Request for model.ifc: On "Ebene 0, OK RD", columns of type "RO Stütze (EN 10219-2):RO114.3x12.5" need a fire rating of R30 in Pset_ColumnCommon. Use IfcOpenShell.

First a look at what the model holds.

```python
import ifcopenshell
import ifcopenshell.util.element

model = ifcopenshell.open("model.ifc")
print(model.schema)
storey = next(s for s in model.by_type("IfcBuildingStorey") if s.Name == "Ebene 0, OK RD")
columns = [e for e in ifcopenshell.util.element.get_decomposition(storey) if e.is_a("IfcColumn")]
seen = {}
for e in columns:
    element_type = ifcopenshell.util.element.get_type(e)
    key = (element_type.Name if element_type != e and element_type else None, ifcopenshell.util.element.get_pset(e, "Pset_ColumnCommon", "FireRating"))
    seen[key] = seen.get(key, 0) + 1
for (name, value), count in sorted(seen.items(), key=str):
    print(count, "x", name, "|", value)
```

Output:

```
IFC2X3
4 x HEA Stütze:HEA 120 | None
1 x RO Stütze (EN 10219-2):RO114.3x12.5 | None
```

```python
import ifcopenshell
import ifcopenshell.api.pset
import ifcopenshell.util.element

model = ifcopenshell.open("model.ifc")

storey = next(s for s in model.by_type("IfcBuildingStorey") if s.Name == "Ebene 0, OK RD")
columns = [e for e in ifcopenshell.util.element.get_decomposition(storey) if e.is_a("IfcColumn")]

count = 0
for e in columns:
    element_type = ifcopenshell.util.element.get_type(e)
    if element_type in (None, e) or element_type.Name != "RO Stütze (EN 10219-2):RO114.3x12.5":
        continue
    # add_pset returns the element's existing set when there is one.
    pset = ifcopenshell.api.pset.add_pset(model, product=e, name="Pset_ColumnCommon")
    ifcopenshell.api.pset.edit_pset(model, pset=pset, properties={"FireRating": "R30"})
    count += 1

print(count, "columns updated")

model.write("model-out.ifc")
```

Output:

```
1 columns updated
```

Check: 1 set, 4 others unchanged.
